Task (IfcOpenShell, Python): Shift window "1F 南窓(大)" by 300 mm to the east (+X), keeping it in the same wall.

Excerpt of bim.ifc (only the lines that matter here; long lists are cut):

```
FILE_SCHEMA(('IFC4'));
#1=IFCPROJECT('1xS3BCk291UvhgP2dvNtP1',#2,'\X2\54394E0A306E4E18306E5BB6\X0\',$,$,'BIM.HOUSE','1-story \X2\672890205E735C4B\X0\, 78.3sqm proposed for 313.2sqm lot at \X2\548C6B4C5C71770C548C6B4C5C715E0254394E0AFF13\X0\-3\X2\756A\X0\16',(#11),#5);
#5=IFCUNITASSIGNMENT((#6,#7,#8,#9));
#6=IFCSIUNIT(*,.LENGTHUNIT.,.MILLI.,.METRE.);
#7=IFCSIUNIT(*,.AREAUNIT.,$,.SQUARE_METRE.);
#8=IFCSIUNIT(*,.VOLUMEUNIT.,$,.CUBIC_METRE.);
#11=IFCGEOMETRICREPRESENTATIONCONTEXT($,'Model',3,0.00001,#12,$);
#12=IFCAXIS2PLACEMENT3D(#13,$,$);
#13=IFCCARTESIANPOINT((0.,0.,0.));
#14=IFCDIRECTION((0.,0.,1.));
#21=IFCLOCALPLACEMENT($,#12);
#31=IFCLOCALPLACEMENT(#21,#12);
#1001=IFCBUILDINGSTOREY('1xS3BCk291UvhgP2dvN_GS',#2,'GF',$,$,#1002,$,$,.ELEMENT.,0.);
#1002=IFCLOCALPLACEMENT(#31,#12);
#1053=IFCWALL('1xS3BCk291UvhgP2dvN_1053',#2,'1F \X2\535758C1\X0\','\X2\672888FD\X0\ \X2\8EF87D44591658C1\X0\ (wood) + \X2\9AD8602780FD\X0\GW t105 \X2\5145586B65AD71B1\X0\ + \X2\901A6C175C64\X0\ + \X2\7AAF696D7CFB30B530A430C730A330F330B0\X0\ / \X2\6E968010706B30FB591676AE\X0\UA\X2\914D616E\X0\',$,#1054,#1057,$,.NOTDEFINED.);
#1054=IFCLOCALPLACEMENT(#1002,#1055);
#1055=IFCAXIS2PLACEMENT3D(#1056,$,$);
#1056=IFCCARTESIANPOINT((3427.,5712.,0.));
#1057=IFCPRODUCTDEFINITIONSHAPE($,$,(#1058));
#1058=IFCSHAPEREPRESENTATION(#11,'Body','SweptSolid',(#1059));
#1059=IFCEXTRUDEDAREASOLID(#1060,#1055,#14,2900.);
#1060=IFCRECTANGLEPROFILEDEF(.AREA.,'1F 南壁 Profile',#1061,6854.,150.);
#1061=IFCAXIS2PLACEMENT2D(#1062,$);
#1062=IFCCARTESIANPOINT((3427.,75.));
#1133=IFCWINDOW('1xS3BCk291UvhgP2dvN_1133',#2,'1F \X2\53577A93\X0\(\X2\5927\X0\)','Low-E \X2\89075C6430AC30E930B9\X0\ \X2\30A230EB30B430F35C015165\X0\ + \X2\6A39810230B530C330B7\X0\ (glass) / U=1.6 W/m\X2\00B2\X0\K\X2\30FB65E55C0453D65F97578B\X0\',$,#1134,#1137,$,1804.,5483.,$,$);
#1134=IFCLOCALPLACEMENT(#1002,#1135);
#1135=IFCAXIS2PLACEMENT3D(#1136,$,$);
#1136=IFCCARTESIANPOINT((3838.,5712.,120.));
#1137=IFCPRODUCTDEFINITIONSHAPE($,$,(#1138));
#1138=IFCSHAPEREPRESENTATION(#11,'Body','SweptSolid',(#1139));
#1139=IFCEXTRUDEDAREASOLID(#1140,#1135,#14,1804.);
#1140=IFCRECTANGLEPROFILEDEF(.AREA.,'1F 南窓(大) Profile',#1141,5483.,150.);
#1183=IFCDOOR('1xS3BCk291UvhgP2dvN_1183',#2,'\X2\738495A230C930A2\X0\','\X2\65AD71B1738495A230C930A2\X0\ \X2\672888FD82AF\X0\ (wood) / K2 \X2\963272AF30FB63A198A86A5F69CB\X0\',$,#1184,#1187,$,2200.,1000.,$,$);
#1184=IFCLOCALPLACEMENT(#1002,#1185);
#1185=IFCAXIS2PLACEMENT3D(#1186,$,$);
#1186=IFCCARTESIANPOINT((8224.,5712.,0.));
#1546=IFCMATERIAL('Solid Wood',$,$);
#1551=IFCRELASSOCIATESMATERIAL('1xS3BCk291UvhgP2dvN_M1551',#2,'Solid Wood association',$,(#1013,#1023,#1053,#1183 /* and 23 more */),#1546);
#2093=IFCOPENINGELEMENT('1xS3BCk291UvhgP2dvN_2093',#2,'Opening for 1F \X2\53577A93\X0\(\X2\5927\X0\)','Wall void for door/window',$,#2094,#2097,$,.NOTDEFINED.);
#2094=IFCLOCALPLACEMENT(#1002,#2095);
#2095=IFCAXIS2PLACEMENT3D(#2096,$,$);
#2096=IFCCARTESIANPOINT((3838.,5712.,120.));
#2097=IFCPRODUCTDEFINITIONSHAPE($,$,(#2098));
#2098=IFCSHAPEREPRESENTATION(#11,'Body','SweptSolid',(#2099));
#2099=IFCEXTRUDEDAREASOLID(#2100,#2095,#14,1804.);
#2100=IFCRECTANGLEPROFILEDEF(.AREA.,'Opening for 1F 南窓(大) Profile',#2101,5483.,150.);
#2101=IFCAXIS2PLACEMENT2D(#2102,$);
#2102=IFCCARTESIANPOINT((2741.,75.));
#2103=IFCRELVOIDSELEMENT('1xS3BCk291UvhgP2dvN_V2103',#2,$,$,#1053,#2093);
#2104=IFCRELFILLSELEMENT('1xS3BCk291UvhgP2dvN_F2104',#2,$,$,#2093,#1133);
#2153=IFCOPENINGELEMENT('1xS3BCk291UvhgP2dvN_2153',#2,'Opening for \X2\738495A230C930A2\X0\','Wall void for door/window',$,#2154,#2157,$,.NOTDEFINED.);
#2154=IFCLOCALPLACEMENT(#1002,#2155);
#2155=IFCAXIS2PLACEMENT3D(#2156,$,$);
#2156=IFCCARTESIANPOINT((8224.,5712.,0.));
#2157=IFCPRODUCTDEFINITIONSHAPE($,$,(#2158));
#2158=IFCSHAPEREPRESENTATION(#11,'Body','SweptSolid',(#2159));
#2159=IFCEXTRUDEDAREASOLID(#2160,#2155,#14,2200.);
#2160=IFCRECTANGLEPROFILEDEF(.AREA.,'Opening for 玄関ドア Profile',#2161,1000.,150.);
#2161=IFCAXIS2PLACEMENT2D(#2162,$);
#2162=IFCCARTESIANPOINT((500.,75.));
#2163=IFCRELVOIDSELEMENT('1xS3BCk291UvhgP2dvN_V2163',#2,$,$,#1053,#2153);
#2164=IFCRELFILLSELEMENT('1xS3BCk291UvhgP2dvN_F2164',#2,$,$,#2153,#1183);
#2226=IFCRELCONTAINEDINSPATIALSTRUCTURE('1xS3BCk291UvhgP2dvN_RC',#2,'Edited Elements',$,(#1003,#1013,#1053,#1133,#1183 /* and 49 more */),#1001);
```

```python
import ifcopenshell
import ifcopenshell.api.geometry
import ifcopenshell.util.placement
import ifcopenshell.util.unit

model = ifcopenshell.open("bim.ifc")
unit_scale = ifcopenshell.util.unit.calculate_unit_scale(model)

window = model.by_guid("1xS3BCk291UvhgP2dvN_1133")
opening = window.FillsVoids[0].RelatingOpeningElement
wall = opening.VoidsElements[0].RelatingBuildingElement

wall_matrix = ifcopenshell.util.placement.get_local_placement(wall.ObjectPlacement)
shift = wall_matrix[:3, 0] * 0.3 / unit_scale
before = ifcopenshell.util.placement.get_local_placement(window.ObjectPlacement)[:3, 3].copy()

# The window is not placed relative to its opening, so move both.
for product in (opening, window):
    matrix = ifcopenshell.util.placement.get_local_placement(product.ObjectPlacement)
    matrix[:3, 3] += shift
    ifcopenshell.api.geometry.edit_object_placement(model, product=product, matrix=matrix, is_si=False)

after = ifcopenshell.util.placement.get_local_placement(window.ObjectPlacement)[:3, 3]
print("window moved by", (after - before).round(3) + 0.0)

model.write("bim_v2.ifc")
```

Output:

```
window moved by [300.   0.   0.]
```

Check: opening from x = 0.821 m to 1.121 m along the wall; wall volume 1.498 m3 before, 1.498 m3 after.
